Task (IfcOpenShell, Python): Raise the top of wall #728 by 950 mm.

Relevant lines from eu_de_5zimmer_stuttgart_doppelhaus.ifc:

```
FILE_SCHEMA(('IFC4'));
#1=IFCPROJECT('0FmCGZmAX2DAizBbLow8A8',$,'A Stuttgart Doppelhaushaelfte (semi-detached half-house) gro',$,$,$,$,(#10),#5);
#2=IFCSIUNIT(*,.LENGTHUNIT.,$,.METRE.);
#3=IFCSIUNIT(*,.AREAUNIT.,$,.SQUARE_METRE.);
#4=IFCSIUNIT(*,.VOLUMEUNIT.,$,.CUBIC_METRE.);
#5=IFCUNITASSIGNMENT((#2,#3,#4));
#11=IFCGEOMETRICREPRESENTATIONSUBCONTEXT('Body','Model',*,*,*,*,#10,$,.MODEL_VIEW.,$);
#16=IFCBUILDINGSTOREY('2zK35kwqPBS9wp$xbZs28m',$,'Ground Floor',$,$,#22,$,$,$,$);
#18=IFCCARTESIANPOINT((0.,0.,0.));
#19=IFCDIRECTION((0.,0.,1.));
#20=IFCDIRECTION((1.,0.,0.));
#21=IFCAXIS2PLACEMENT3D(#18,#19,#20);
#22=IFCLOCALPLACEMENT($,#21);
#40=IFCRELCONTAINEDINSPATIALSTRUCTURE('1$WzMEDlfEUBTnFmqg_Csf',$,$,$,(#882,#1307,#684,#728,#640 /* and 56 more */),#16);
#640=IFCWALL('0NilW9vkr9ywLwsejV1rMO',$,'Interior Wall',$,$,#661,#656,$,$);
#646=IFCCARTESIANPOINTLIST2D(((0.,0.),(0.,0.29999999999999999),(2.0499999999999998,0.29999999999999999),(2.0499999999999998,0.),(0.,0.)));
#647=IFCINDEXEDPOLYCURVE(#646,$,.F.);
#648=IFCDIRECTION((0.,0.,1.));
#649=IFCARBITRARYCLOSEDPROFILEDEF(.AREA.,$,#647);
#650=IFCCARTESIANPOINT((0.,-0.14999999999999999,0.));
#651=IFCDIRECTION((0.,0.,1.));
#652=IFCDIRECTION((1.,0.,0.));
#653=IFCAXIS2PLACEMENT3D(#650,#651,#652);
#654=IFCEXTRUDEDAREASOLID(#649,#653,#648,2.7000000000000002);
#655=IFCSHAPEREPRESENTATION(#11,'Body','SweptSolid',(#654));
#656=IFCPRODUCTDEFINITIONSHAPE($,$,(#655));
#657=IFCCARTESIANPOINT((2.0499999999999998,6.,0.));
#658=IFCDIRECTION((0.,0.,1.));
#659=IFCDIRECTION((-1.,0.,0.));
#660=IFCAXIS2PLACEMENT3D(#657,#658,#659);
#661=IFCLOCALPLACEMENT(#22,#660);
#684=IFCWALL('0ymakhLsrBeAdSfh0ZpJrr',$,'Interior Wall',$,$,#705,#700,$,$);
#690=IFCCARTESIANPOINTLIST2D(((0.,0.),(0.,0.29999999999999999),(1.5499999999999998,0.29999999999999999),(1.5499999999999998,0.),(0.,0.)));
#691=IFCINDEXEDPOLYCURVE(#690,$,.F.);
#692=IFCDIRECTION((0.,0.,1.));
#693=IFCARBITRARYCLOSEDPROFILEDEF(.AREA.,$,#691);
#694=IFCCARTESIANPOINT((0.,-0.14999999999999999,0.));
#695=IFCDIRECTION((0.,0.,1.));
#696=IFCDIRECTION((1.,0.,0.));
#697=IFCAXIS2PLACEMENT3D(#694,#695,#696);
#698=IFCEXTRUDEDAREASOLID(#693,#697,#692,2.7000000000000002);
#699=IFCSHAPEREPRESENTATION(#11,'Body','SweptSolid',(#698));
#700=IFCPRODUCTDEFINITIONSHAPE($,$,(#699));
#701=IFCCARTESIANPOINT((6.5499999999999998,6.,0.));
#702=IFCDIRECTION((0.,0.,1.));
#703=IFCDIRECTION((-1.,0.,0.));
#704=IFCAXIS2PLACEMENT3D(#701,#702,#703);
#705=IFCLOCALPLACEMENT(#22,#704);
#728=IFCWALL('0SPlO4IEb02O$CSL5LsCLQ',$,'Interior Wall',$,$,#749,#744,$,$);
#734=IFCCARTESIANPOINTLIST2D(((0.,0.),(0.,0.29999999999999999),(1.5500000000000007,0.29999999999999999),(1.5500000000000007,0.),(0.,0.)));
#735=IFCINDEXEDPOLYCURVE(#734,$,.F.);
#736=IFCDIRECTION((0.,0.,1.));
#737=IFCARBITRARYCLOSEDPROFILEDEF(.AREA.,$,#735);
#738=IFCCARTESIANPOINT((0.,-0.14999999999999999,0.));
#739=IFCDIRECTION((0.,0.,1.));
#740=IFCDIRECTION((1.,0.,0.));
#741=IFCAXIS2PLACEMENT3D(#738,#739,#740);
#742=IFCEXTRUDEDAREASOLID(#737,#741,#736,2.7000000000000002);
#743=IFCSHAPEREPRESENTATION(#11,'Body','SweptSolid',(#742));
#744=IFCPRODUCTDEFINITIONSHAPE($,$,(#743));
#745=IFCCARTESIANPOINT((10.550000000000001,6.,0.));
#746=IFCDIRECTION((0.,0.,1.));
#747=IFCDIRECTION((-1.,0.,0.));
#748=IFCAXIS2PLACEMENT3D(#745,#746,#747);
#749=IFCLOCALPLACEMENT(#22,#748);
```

```python
import ifcopenshell
import ifcopenshell.geom
import ifcopenshell.util.representation
import ifcopenshell.util.shape
import ifcopenshell.util.unit

model = ifcopenshell.open("eu_de_5zimmer_stuttgart_doppelhaus.ifc")
unit_scale = ifcopenshell.util.unit.calculate_unit_scale(model)
settings = ifcopenshell.geom.settings()


def volume(element):
    """Net volume in cubic metres, openings subtracted."""
    shape = ifcopenshell.geom.create_shape(settings, element)
    return ifcopenshell.util.shape.get_volume(shape.geometry)


wall = model.by_id(728)
before = volume(wall)

body = ifcopenshell.util.representation.get_representation(wall, "Model", "Body")
solid = body.Items[0]
old_height = solid.Depth
solid.Depth += 0.95 / unit_scale
after = volume(wall)

print(f"height {old_height:g} -> {solid.Depth:g}, volume {before:.3f} -> {after:.3f} m3")

model.write("eu_de_5zimmer_stuttgart_doppelhaus_updated.ifc")
```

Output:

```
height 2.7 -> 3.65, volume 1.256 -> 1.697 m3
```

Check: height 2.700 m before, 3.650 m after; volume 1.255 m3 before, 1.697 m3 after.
